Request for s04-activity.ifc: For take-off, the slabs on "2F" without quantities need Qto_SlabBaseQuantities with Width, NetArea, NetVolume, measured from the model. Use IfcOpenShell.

First a look at what the model holds.

```python
import ifcopenshell
import ifcopenshell.util.element
import ifcopenshell.util.unit

model = ifcopenshell.open("s04-activity.ifc")
print(model.schema)
for unit_type in ("LENGTHUNIT", "AREAUNIT", "VOLUMEUNIT"):
    print(unit_type, ifcopenshell.util.unit.calculate_unit_scale(model, unit_type))
storey = next(s for s in model.by_type("IfcBuildingStorey") if s.Name == "2F")
slabs = [e for e in ifcopenshell.util.element.get_decomposition(storey) if e.is_a("IfcSlab")]
for e in sorted(slabs, key=lambda e: e.id()):
    print(e.id(), e.is_a(), e.Name, list(ifcopenshell.util.element.get_psets(e, qtos_only=True)), sep=" | ")
```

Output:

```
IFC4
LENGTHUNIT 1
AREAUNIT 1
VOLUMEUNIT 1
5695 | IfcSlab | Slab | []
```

```python
import ifcopenshell
import ifcopenshell.api.pset
import ifcopenshell.geom
import ifcopenshell.util.element
import ifcopenshell.util.shape
import ifcopenshell.util.unit

model = ifcopenshell.open("s04-activity.ifc")
unit_scale = ifcopenshell.util.unit.calculate_unit_scale(model)
area_scale = ifcopenshell.util.unit.calculate_unit_scale(model, "AREAUNIT")
volume_scale = ifcopenshell.util.unit.calculate_unit_scale(model, "VOLUMEUNIT")
settings = ifcopenshell.geom.settings()

storey = next(s for s in model.by_type("IfcBuildingStorey") if s.Name == "2F")
slabs = [e for e in ifcopenshell.util.element.get_decomposition(storey) if e.is_a("IfcSlab")]

for e in sorted(slabs, key=lambda e: e.id()):
    if ifcopenshell.util.element.get_psets(e, qtos_only=True, should_inherit=False):
        continue
    # Geometry comes back in metres, in the element's own axes.
    shape = ifcopenshell.geom.create_shape(settings, e)
    values = {
        "Width": ifcopenshell.util.shape.get_z(shape.geometry) / unit_scale,
        "NetArea": ifcopenshell.util.shape.get_footprint_area(shape.geometry) / area_scale,
        "NetVolume": ifcopenshell.util.shape.get_volume(shape.geometry) / volume_scale,
    }
    qto = ifcopenshell.api.pset.add_qto(model, product=e, name="Qto_SlabBaseQuantities")
    ifcopenshell.api.pset.edit_qto(model, qto=qto, properties=values)
    print(e.id(), {k: round(v, 3) for k, v in values.items()})

model.write("s04-activity_rev.ifc")
```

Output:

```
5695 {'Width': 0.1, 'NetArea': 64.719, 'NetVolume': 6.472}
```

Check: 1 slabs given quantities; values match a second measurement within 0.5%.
